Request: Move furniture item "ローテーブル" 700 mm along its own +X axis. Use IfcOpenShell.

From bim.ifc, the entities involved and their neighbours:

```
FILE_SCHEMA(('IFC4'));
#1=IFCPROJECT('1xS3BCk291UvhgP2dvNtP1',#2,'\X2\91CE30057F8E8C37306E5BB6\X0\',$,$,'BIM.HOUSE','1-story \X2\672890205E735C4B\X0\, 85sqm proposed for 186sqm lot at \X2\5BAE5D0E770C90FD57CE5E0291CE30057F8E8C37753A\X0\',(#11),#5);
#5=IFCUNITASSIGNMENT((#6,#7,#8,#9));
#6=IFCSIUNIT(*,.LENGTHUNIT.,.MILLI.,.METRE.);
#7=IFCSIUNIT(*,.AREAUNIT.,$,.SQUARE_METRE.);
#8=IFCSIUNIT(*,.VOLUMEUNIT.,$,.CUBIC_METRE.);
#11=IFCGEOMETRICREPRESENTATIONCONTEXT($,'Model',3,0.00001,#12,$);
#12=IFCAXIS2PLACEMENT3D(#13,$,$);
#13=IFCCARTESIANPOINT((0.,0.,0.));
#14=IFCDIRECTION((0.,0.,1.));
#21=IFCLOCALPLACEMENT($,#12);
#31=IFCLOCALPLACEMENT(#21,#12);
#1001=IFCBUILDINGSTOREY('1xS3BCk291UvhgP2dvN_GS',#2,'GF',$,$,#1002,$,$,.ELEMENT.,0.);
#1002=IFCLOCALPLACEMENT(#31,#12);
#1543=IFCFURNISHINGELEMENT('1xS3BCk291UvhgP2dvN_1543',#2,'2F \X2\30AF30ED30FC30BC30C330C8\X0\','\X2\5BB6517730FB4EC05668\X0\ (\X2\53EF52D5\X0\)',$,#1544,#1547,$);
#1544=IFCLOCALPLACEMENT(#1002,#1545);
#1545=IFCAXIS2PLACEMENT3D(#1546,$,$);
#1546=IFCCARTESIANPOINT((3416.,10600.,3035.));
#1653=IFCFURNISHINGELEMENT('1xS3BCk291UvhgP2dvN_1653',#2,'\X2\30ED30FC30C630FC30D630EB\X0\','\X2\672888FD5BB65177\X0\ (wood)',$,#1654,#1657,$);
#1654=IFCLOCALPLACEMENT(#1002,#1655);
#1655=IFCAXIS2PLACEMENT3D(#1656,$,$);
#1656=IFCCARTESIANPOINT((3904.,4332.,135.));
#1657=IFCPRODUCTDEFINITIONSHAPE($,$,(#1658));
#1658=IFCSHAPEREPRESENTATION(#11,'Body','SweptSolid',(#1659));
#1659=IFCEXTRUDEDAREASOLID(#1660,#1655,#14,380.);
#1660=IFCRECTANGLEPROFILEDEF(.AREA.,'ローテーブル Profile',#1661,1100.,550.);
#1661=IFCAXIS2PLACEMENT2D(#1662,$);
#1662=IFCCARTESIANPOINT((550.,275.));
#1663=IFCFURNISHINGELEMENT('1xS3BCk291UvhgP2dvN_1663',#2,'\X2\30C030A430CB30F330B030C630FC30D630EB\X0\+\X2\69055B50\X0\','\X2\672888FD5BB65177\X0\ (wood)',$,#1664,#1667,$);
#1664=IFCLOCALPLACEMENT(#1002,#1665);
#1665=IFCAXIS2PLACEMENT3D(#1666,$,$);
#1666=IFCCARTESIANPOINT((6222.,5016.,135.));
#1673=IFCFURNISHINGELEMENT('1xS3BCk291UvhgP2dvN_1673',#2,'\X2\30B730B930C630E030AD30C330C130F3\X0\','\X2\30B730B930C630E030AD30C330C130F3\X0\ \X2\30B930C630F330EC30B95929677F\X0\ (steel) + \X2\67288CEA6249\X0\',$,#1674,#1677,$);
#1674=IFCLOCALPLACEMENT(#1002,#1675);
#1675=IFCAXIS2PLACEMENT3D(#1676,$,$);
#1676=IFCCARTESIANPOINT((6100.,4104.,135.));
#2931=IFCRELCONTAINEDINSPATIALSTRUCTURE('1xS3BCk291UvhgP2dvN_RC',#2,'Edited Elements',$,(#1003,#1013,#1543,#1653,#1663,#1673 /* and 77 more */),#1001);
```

```python
import ifcopenshell
import ifcopenshell.api.geometry
import ifcopenshell.util.placement
import ifcopenshell.util.unit

model = ifcopenshell.open("bim.ifc")
unit_scale = ifcopenshell.util.unit.calculate_unit_scale(model)

item = model.by_guid("1xS3BCk291UvhgP2dvN_1653")
matrix = ifcopenshell.util.placement.get_local_placement(item.ObjectPlacement)
matrix[:3, 3] += matrix[:3, 0] * 0.7 / unit_scale
ifcopenshell.api.geometry.edit_object_placement(model, product=item, matrix=matrix, is_si=False)

print(ifcopenshell.util.placement.get_local_placement(item.ObjectPlacement).round(3) + 0.0)

model.write("bim_v2.ifc")
```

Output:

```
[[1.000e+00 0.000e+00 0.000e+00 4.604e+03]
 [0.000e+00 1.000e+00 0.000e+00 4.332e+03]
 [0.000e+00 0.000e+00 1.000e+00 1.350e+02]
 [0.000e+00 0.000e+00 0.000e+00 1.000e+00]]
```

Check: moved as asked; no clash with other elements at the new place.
